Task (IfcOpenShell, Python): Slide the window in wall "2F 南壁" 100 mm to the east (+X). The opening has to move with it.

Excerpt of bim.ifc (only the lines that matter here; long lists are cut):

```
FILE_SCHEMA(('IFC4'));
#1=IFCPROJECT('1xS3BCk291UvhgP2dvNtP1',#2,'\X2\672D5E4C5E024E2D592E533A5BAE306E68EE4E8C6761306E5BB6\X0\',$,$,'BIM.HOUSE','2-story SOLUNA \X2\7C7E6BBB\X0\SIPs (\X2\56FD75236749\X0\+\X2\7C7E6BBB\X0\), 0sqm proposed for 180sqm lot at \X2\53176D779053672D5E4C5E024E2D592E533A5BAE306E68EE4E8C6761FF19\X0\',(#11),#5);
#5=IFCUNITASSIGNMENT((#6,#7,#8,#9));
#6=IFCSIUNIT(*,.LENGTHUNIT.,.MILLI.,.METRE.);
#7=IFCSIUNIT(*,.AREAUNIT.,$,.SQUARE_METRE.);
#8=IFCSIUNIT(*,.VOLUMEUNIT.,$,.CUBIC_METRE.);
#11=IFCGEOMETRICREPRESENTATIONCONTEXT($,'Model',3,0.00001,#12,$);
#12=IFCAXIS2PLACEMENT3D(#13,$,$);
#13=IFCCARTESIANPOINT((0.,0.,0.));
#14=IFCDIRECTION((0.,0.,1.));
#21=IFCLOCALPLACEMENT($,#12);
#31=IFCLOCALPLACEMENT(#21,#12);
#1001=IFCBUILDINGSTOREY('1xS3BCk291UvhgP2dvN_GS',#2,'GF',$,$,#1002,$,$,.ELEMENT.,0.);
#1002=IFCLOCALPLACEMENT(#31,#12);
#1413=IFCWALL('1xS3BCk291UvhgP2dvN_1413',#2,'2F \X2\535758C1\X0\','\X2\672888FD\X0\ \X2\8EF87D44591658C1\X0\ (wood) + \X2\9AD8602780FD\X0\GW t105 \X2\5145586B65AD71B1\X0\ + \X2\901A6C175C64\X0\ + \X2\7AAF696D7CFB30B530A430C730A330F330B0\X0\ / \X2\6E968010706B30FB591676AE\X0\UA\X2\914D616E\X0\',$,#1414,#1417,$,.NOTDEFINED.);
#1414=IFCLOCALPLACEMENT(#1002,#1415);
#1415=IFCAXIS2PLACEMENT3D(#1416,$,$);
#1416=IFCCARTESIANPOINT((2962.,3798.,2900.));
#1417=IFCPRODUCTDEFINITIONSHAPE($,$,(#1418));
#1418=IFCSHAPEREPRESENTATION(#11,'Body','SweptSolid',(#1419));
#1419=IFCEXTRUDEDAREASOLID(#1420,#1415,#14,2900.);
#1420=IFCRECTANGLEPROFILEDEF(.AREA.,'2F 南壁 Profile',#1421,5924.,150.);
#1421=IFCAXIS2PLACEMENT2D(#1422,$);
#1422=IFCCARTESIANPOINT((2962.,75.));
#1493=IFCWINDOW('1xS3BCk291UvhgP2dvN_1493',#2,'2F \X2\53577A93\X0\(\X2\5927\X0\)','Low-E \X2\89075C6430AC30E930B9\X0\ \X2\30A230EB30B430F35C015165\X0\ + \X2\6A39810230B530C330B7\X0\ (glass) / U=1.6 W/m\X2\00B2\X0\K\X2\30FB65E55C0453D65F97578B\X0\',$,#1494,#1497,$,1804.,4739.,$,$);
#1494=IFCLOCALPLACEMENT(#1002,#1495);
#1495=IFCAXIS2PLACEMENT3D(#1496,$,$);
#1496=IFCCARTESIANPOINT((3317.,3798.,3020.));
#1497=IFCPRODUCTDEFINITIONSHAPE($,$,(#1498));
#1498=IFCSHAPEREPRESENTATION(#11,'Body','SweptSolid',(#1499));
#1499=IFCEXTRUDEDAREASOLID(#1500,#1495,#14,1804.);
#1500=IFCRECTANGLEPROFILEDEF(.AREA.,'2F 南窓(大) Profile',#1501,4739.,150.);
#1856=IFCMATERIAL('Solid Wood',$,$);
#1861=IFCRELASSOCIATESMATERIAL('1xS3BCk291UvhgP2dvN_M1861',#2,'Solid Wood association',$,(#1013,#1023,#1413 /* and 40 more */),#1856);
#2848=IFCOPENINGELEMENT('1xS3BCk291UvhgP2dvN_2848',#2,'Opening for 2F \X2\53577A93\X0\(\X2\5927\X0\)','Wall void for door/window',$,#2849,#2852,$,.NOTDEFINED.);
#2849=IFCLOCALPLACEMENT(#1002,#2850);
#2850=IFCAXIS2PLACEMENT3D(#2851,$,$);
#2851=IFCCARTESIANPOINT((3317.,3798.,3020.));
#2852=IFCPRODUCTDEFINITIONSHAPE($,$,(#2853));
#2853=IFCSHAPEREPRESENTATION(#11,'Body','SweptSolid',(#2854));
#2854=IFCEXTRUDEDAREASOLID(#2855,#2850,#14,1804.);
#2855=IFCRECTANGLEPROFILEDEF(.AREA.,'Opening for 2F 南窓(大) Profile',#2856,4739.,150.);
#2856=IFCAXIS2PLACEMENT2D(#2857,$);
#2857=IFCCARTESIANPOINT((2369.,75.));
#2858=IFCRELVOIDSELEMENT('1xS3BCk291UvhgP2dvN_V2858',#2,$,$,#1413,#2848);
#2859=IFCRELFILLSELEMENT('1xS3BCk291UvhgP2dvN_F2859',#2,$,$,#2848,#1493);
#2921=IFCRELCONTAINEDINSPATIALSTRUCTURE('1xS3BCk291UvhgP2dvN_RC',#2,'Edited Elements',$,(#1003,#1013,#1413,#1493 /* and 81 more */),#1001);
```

```python
import ifcopenshell
import ifcopenshell.api.geometry
import ifcopenshell.util.placement
import ifcopenshell.util.unit

model = ifcopenshell.open("bim.ifc")
unit_scale = ifcopenshell.util.unit.calculate_unit_scale(model)

window = model.by_guid("1xS3BCk291UvhgP2dvN_1493")
opening = window.FillsVoids[0].RelatingOpeningElement
wall = opening.VoidsElements[0].RelatingBuildingElement

wall_matrix = ifcopenshell.util.placement.get_local_placement(wall.ObjectPlacement)
shift = wall_matrix[:3, 0] * 0.1 / unit_scale
before = ifcopenshell.util.placement.get_local_placement(window.ObjectPlacement)[:3, 3].copy()

# The window is not placed relative to its opening, so move both.
for product in (opening, window):
    matrix = ifcopenshell.util.placement.get_local_placement(product.ObjectPlacement)
    matrix[:3, 3] += shift
    ifcopenshell.api.geometry.edit_object_placement(model, product=product, matrix=matrix, is_si=False)

after = ifcopenshell.util.placement.get_local_placement(window.ObjectPlacement)[:3, 3]
print("window moved by", (after - before).round(3) + 0.0)

model.write("bim-out.ifc")
```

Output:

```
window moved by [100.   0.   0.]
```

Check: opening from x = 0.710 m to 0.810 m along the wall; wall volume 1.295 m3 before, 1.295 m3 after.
